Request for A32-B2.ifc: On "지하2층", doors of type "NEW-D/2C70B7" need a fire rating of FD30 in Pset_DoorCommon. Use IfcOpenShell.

First a look at what the model holds.

```python
import ifcopenshell
import ifcopenshell.util.element

model = ifcopenshell.open("A32-B2.ifc")
print(model.schema)
storey = next(s for s in model.by_type("IfcBuildingStorey") if s.Name == "지하2층")
doors = [e for e in ifcopenshell.util.element.get_decomposition(storey) if e.is_a("IfcDoor")]
seen = {}
for e in doors:
    element_type = ifcopenshell.util.element.get_type(e)
    key = (element_type.Name if element_type != e and element_type else None, ifcopenshell.util.element.get_pset(e, "Pset_DoorCommon", "FireRating"))
    seen[key] = seen.get(key, 0) + 1
for (name, value), count in sorted(seen.items(), key=str):
    print(count, "x", name, "|", value)
```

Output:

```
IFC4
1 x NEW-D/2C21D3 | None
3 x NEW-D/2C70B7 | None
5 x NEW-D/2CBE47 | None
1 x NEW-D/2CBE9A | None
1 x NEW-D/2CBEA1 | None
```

```python
import ifcopenshell
import ifcopenshell.api.pset
import ifcopenshell.util.element

model = ifcopenshell.open("A32-B2.ifc")

storey = next(s for s in model.by_type("IfcBuildingStorey") if s.Name == "지하2층")
doors = [e for e in ifcopenshell.util.element.get_decomposition(storey) if e.is_a("IfcDoor")]

count = 0
for e in doors:
    element_type = ifcopenshell.util.element.get_type(e)
    if element_type in (None, e) or element_type.Name != "NEW-D/2C70B7":
        continue
    # add_pset returns the element's existing set when there is one.
    pset = ifcopenshell.api.pset.add_pset(model, product=e, name="Pset_DoorCommon")
    ifcopenshell.api.pset.edit_pset(model, pset=pset, properties={"FireRating": "FD30"})
    count += 1

print(count, "doors updated")

model.write("A32-B2_v2.ifc")
```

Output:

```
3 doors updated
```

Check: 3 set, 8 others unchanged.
